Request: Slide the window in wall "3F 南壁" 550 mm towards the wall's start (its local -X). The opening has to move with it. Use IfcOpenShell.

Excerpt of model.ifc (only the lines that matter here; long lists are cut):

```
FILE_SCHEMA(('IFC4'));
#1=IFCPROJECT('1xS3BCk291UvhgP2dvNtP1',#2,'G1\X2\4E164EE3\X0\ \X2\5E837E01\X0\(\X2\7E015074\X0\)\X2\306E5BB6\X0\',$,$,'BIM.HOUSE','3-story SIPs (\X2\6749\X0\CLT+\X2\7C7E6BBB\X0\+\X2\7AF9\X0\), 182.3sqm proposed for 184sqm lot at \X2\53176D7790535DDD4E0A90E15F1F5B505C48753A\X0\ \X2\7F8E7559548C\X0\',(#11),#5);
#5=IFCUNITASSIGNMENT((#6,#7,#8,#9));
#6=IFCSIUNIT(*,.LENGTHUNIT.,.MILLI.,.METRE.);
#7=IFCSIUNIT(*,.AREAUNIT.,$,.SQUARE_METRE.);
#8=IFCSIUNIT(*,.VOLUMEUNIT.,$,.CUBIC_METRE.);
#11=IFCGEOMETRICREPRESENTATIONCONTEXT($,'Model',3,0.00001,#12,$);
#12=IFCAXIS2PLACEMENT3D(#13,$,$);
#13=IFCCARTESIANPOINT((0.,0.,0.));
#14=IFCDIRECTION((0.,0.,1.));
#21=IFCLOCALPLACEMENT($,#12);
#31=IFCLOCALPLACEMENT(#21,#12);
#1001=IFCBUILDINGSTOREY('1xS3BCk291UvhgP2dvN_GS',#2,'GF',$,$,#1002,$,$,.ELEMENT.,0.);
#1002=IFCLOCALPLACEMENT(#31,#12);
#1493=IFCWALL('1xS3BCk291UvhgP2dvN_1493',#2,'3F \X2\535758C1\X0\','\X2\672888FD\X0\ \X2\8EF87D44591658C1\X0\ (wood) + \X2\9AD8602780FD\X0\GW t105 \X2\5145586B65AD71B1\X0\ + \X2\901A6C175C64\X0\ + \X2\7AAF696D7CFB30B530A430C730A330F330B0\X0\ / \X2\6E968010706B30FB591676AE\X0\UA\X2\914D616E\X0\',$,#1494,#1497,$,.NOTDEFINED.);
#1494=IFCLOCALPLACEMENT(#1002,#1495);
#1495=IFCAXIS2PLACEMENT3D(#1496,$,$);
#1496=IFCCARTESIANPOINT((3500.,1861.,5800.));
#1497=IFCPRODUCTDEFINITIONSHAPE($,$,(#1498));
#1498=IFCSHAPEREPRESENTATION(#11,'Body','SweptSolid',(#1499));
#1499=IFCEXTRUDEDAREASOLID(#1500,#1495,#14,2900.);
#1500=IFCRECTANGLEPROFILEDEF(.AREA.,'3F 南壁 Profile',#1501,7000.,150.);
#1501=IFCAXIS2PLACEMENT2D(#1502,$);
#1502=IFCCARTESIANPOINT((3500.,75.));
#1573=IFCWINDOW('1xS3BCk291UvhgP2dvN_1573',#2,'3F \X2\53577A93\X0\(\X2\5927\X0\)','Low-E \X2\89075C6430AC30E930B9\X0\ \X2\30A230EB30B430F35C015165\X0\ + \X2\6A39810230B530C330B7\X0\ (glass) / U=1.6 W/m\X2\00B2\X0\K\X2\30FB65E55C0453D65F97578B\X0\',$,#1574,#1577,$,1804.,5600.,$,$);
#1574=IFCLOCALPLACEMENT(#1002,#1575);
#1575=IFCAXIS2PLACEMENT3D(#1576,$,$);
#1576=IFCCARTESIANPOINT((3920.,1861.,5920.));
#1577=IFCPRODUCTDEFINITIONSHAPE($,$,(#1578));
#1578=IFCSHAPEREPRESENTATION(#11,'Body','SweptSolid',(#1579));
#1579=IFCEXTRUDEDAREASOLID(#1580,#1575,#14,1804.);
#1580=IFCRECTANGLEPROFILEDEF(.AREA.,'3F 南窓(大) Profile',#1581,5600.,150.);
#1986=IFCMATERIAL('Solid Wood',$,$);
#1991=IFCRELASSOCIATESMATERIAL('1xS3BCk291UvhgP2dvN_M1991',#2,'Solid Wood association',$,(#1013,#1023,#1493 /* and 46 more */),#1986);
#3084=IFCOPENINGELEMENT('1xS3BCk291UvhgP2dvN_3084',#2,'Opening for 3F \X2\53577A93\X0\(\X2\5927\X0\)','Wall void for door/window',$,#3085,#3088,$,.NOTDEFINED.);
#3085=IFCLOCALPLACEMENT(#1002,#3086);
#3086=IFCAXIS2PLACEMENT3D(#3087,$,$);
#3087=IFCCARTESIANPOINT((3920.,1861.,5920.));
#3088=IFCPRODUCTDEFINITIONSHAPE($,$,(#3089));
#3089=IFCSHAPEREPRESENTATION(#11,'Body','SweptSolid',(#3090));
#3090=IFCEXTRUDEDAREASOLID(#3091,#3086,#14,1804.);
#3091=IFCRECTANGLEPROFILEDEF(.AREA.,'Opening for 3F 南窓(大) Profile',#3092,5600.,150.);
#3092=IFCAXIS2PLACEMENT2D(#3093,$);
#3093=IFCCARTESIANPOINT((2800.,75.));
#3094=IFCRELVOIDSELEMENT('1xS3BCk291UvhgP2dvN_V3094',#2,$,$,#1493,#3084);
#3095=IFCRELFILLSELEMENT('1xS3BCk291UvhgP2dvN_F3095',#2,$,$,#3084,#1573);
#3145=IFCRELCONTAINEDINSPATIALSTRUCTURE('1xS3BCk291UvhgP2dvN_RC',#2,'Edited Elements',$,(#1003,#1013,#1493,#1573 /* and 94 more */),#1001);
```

```python
import ifcopenshell
import ifcopenshell.api.geometry
import ifcopenshell.util.placement
import ifcopenshell.util.unit

model = ifcopenshell.open("model.ifc")
unit_scale = ifcopenshell.util.unit.calculate_unit_scale(model)

window = model.by_guid("1xS3BCk291UvhgP2dvN_1573")
opening = window.FillsVoids[0].RelatingOpeningElement
wall = opening.VoidsElements[0].RelatingBuildingElement

wall_matrix = ifcopenshell.util.placement.get_local_placement(wall.ObjectPlacement)
shift = wall_matrix[:3, 0] * -0.55 / unit_scale
before = ifcopenshell.util.placement.get_local_placement(window.ObjectPlacement)[:3, 3].copy()

# The window is not placed relative to its opening, so move both.
for product in (opening, window):
    matrix = ifcopenshell.util.placement.get_local_placement(product.ObjectPlacement)
    matrix[:3, 3] += shift
    ifcopenshell.api.geometry.edit_object_placement(model, product=product, matrix=matrix, is_si=False)

after = ifcopenshell.util.placement.get_local_placement(window.ObjectPlacement)[:3, 3]
print("window moved by", (after - before).round(3) + 0.0)

model.write("model_rev.ifc")
```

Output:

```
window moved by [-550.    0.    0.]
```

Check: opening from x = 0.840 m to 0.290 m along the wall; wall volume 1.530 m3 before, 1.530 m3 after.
